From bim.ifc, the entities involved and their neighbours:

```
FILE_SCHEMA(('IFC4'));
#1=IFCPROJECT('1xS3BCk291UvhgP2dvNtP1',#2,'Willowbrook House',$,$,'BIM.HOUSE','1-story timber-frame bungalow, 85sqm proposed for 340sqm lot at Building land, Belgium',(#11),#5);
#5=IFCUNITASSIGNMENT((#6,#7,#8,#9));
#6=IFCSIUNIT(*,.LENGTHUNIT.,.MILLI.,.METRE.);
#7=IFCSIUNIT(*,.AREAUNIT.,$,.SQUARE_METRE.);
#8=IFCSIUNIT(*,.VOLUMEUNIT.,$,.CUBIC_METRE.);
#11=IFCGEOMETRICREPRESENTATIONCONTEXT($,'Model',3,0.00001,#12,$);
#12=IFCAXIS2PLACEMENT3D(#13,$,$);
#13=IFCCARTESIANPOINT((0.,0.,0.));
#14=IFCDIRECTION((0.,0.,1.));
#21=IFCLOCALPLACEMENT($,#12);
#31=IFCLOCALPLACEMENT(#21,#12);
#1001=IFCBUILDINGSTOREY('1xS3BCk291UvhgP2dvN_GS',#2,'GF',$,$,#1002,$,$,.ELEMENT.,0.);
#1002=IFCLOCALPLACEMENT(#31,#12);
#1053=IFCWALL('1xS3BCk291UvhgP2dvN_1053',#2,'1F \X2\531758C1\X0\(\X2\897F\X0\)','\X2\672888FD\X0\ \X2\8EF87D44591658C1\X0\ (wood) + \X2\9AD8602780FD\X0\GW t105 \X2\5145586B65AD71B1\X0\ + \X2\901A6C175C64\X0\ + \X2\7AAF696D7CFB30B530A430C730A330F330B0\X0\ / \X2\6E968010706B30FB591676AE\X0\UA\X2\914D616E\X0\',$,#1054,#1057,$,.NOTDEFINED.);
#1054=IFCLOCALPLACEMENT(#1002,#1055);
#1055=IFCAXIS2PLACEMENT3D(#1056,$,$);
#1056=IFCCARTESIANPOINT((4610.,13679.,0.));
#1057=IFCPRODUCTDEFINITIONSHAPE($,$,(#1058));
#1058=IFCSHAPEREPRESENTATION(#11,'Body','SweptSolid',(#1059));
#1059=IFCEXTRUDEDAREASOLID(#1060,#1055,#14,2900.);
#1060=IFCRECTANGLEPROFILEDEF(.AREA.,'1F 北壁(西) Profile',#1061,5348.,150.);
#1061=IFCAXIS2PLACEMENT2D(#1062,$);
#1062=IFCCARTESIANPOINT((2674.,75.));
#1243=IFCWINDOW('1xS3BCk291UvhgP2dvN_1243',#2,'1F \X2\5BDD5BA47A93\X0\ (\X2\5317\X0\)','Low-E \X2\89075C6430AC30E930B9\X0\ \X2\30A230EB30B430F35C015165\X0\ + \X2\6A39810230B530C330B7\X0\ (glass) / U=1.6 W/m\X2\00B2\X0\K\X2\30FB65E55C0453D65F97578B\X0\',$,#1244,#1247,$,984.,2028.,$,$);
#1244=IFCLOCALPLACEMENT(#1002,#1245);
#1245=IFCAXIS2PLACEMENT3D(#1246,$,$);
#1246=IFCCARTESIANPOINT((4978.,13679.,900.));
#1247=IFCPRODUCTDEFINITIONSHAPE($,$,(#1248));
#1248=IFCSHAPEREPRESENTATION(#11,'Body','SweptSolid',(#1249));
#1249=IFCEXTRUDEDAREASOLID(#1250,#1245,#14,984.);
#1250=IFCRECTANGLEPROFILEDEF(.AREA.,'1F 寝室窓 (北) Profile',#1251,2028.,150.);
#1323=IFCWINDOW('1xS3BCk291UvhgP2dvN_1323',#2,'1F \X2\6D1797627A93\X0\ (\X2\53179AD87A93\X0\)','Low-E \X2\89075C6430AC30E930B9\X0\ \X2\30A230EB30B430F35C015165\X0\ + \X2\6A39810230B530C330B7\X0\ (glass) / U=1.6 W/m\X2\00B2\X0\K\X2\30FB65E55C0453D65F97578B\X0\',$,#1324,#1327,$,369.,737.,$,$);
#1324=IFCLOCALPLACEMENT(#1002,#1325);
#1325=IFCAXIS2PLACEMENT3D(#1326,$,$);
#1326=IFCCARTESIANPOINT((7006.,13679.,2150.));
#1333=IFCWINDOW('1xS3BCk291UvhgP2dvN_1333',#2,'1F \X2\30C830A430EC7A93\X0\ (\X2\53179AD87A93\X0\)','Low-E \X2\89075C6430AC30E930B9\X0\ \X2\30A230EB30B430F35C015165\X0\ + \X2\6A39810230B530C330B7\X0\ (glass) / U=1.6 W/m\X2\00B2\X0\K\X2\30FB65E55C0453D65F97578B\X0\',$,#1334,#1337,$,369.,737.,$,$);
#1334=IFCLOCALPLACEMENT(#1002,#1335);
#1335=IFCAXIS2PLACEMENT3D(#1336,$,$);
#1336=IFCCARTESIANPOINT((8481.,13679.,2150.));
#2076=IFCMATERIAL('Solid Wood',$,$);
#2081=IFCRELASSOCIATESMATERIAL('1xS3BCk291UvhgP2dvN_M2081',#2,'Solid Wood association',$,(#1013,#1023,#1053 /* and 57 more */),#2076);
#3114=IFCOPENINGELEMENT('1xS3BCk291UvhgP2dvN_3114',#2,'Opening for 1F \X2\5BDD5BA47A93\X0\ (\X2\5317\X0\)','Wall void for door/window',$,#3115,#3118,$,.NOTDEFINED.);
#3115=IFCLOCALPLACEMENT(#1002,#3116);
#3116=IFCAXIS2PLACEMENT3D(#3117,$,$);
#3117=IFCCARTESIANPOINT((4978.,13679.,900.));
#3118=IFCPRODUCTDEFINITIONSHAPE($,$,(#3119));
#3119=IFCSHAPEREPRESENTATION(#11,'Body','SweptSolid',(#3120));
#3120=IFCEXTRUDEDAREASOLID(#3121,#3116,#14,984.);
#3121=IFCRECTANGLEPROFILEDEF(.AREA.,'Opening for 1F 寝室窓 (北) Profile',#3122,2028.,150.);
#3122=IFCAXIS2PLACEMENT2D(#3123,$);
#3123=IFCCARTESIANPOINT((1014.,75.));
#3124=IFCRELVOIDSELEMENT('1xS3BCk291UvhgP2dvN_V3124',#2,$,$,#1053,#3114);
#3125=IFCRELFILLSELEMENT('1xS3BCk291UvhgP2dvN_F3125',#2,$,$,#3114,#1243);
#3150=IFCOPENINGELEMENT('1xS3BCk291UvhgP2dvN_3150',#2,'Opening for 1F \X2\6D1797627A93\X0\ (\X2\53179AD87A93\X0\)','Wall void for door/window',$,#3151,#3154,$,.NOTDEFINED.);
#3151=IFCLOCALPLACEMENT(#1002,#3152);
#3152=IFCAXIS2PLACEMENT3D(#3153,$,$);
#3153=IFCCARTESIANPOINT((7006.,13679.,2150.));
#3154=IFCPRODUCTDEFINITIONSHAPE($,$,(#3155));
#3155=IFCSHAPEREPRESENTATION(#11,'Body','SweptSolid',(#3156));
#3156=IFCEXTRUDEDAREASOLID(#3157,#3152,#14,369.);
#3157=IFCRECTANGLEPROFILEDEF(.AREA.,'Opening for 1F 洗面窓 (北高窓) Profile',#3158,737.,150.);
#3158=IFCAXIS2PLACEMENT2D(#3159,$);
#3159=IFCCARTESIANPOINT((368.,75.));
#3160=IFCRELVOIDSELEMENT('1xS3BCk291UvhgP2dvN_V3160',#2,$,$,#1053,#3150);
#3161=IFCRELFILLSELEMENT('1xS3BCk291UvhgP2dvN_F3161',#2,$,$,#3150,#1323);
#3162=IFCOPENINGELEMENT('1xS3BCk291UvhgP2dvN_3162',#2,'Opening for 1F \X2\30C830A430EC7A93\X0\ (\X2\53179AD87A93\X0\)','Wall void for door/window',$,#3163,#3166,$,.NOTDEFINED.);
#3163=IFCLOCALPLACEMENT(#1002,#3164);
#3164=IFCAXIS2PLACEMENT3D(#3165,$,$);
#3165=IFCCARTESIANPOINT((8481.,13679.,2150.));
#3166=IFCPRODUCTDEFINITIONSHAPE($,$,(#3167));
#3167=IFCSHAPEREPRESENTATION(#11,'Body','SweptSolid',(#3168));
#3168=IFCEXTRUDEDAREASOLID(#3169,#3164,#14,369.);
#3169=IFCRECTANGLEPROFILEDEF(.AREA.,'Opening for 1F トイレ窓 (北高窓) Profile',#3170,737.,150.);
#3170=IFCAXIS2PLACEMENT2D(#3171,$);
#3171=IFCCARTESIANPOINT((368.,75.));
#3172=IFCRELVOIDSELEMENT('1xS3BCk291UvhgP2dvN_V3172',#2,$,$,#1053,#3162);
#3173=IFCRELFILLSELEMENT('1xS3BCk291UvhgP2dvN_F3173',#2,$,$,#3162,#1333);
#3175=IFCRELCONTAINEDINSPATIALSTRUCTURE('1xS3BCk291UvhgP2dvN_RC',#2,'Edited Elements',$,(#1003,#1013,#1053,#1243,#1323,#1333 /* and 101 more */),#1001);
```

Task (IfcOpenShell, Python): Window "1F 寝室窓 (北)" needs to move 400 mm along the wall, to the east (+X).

```python
import ifcopenshell
import ifcopenshell.api.geometry
import ifcopenshell.util.placement

model = ifcopenshell.open("bim.ifc")

window = model.by_id(1243)
opening = window.FillsVoids[0].RelatingOpeningElement
wall = opening.VoidsElements[0].RelatingBuildingElement

wall_matrix = ifcopenshell.util.placement.get_local_placement(wall.ObjectPlacement)
shift = wall_matrix[:3, 0] * 400.0
before = ifcopenshell.util.placement.get_local_placement(window.ObjectPlacement)[:3, 3].copy()

# The window is not placed relative to its opening, so move both.
for product in (opening, window):
    matrix = ifcopenshell.util.placement.get_local_placement(product.ObjectPlacement)
    matrix[:3, 3] += shift
    ifcopenshell.api.geometry.edit_object_placement(model, product=product, matrix=matrix, is_si=False)

after = ifcopenshell.util.placement.get_local_placement(window.ObjectPlacement)[:3, 3]
print("window moved by", (after - before).round(3) + 0.0)

model.write("bim_updated.ifc")
```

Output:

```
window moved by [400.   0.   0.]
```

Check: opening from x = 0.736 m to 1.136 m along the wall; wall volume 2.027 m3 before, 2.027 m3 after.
